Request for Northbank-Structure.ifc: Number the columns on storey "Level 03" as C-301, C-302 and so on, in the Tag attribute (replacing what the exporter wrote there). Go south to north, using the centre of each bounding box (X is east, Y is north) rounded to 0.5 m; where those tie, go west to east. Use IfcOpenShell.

First a look at what the model holds.

```python
import ifcopenshell
import ifcopenshell.util.element
import ifcopenshell.util.placement

model = ifcopenshell.open("Northbank-Structure.ifc")
print(model.schema)
storey = next(s for s in model.by_type("IfcBuildingStorey") if s.Name == "Level 03")
columns = [e for e in ifcopenshell.util.element.get_decomposition(storey) if e.is_a("IfcColumn")]
for e in sorted(columns, key=lambda e: e.id()):
    origin = ifcopenshell.util.placement.get_local_placement(e.ObjectPlacement)[:3, 3]
    print(e.id(), e.Tag, e.Name, origin.round(2) + 0.0, sep=" | ")
```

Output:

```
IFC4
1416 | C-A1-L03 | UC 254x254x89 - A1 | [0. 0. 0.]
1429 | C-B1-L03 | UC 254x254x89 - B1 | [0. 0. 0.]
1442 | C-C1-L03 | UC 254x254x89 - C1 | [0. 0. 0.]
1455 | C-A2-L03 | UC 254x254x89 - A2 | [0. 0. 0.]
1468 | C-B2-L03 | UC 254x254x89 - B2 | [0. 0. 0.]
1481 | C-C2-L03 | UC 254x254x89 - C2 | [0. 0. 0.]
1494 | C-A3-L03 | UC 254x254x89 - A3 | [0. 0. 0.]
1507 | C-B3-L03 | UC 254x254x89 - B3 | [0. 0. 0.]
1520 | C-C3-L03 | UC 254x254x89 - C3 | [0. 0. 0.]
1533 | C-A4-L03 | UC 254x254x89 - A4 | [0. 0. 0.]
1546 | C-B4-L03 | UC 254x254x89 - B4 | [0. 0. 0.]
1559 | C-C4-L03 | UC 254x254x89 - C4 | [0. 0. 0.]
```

```python
import ifcopenshell
import ifcopenshell.geom
import ifcopenshell.util.element
import ifcopenshell.util.shape

model = ifcopenshell.open("Northbank-Structure.ifc")
settings = ifcopenshell.geom.settings()
settings.set("use-world-coords", True)


def centre(element):
    shape = ifcopenshell.geom.create_shape(settings, element)
    return ifcopenshell.util.shape.get_bbox_centroid(shape.geometry)


storey = next(s for s in model.by_type("IfcBuildingStorey") if s.Name == "Level 03")
columns = [e for e in ifcopenshell.util.element.get_decomposition(storey) if e.is_a("IfcColumn")]

# Insertion points can sit at a corner or the storey origin, so sort by the geometry (in metres).
centres = {e: centre(e) for e in columns}
columns.sort(key=lambda e: (round(centres[e][1] / 0.5), centres[e][0]))

for i, e in enumerate(columns, start=1):
    number = f"C-3{i:02d}"
    e.Tag = number
    print(e.id(), number)

model.write("Northbank-Structure_rev.ifc")
```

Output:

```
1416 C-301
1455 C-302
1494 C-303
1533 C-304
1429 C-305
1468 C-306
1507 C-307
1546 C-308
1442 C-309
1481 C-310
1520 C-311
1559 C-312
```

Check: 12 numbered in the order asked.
